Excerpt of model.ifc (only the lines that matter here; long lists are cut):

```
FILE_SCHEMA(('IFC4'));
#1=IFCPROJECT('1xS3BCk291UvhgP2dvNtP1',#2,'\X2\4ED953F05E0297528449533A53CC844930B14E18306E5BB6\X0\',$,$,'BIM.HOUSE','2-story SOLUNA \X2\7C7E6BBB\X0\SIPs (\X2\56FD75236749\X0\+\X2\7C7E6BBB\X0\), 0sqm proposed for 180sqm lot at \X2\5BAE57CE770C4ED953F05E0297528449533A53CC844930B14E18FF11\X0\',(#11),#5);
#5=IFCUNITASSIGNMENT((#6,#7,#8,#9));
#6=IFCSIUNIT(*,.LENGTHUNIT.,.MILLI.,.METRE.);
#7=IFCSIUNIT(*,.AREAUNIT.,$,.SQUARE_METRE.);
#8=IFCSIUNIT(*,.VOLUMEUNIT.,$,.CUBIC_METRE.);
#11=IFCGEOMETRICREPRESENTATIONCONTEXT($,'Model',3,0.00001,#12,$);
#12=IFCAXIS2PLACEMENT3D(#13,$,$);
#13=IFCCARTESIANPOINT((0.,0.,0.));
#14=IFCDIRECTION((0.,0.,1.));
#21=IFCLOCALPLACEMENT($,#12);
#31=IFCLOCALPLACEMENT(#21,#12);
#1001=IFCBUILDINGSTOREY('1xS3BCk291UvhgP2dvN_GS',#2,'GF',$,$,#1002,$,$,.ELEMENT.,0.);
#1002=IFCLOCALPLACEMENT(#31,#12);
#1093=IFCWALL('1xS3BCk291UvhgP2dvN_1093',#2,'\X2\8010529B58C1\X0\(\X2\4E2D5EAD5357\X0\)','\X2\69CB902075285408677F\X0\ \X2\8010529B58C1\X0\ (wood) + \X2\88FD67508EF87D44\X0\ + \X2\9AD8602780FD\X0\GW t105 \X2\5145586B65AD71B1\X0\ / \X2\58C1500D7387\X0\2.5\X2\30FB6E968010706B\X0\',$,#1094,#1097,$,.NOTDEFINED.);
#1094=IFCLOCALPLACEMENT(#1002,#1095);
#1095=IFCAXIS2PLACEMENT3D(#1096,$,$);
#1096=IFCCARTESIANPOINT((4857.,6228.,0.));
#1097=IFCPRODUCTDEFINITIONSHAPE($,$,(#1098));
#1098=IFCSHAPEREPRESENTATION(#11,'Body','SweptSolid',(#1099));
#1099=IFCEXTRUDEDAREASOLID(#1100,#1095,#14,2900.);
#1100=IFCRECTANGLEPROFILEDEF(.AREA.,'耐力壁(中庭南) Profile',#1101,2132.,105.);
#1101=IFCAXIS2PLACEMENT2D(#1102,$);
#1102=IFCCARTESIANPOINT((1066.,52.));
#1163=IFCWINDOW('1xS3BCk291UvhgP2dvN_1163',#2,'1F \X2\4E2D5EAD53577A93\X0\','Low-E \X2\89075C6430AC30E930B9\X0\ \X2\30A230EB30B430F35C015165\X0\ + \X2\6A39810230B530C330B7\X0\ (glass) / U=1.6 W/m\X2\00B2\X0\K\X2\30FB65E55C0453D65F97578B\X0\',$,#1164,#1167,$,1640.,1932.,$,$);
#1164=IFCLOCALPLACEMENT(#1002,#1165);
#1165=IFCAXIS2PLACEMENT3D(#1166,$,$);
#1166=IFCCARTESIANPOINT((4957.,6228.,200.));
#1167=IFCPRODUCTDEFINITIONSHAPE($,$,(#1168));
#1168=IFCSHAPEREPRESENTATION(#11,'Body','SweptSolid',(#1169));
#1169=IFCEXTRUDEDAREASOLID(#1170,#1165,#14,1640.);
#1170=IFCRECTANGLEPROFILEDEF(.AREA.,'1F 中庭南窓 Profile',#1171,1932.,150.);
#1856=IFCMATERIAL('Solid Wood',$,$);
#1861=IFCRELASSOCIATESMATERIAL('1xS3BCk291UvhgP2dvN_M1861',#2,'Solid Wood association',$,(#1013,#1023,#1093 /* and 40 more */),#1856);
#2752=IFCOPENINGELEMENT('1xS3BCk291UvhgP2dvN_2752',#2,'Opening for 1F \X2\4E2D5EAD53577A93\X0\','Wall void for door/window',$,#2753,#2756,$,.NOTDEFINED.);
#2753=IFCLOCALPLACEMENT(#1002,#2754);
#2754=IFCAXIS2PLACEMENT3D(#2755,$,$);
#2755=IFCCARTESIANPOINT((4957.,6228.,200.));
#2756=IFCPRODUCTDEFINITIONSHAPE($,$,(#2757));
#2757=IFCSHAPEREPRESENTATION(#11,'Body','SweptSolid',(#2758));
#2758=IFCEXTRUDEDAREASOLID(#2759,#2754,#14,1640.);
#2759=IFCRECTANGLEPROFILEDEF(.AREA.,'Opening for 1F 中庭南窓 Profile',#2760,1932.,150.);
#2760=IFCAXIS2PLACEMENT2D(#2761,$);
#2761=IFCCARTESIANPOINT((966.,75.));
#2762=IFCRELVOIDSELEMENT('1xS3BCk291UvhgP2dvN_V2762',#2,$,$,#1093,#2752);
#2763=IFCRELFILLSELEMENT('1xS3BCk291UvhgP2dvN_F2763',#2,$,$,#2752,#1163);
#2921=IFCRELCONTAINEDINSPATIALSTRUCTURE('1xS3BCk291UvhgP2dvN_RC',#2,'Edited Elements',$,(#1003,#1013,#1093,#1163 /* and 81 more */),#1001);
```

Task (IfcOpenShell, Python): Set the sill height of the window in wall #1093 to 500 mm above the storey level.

```python
import numpy as np
import ifcopenshell
import ifcopenshell.api.geometry
import ifcopenshell.geom
import ifcopenshell.util.element
import ifcopenshell.util.placement
import ifcopenshell.util.shape
import ifcopenshell.util.unit

model = ifcopenshell.open("model.ifc")
unit_scale = ifcopenshell.util.unit.calculate_unit_scale(model)

window = model.by_guid("1xS3BCk291UvhgP2dvN_1163")
opening = window.FillsVoids[0].RelatingOpeningElement
storey = ifcopenshell.util.element.get_container(window, ifc_class="IfcBuildingStorey")
level = ifcopenshell.util.placement.get_local_placement(storey.ObjectPlacement)[2, 3]

# The opening's origin need not be at the sill, so measure its lowest point.
shape = ifcopenshell.geom.create_shape(ifcopenshell.geom.settings(), opening)
bottom = ifcopenshell.util.shape.get_shape_bottom_elevation(shape, shape.geometry) / unit_scale
dz = level + 500.0 - bottom

shift = np.array([0.0, 0.0, dz])
# The window is not placed relative to its opening, so move both.
for product in (opening, window):
    matrix = ifcopenshell.util.placement.get_local_placement(product.ObjectPlacement)
    matrix[:3, 3] += shift
    ifcopenshell.api.geometry.edit_object_placement(model, product=product, matrix=matrix, is_si=False)

print(f"moved by {dz * unit_scale:+.3f} m")

model.write("model_v2.ifc")
```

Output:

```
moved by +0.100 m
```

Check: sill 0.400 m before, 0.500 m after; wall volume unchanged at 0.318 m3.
